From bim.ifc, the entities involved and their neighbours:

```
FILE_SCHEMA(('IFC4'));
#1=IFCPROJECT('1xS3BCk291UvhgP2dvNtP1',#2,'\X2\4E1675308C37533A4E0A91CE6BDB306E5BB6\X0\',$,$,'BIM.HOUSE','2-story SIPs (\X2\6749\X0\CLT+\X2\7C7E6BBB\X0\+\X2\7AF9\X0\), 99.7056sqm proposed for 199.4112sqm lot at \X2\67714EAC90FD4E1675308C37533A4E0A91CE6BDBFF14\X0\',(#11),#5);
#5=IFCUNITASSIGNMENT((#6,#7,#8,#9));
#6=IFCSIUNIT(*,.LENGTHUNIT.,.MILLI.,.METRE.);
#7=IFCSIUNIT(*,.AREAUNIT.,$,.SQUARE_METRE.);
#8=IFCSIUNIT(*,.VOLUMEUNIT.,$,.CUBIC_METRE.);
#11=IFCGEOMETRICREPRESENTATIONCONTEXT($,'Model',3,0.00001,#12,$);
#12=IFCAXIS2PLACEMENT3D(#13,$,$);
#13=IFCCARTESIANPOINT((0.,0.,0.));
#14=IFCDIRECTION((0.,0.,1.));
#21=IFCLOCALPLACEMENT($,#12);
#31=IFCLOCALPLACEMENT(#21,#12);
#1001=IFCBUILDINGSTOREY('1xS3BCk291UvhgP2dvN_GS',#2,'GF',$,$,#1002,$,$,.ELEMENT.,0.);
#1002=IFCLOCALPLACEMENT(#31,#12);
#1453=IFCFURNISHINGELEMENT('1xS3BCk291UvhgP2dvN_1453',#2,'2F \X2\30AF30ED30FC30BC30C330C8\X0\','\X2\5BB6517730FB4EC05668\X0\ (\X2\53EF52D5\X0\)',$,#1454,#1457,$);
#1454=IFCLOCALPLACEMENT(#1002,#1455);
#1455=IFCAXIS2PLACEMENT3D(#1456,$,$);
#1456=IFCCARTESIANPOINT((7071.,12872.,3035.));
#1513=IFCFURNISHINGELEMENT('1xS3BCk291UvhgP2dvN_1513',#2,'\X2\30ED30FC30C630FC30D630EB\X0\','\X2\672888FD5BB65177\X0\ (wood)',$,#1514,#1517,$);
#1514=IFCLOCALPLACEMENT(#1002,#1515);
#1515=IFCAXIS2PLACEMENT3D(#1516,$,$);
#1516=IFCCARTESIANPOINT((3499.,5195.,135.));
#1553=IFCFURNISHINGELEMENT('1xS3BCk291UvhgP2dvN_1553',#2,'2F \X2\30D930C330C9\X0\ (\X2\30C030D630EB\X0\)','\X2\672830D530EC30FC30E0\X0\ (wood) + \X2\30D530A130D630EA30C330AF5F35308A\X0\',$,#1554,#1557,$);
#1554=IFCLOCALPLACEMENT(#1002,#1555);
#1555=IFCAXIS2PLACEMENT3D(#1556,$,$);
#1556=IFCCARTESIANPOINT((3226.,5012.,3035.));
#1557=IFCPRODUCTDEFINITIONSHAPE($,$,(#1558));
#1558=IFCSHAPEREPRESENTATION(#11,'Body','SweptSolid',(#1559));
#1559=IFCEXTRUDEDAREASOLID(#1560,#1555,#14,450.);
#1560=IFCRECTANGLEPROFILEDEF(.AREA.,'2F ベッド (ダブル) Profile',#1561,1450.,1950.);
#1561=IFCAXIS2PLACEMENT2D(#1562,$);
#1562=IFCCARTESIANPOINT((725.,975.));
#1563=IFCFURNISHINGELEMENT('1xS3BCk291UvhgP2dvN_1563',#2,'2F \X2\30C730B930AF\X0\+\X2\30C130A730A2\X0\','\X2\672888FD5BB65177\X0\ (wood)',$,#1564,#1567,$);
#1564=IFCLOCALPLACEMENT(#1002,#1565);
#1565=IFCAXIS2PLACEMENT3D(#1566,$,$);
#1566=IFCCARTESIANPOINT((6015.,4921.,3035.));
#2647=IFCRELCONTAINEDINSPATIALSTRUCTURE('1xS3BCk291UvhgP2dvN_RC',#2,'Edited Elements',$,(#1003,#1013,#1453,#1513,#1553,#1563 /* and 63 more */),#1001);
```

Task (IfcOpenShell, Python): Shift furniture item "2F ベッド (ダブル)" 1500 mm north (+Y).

```python
import ifcopenshell
import ifcopenshell.api.geometry
import ifcopenshell.util.placement

model = ifcopenshell.open("bim.ifc")

item = model.by_id(1553)
matrix = ifcopenshell.util.placement.get_local_placement(item.ObjectPlacement)
matrix[1, 3] += 1500.0
ifcopenshell.api.geometry.edit_object_placement(model, product=item, matrix=matrix, is_si=False)

print(ifcopenshell.util.placement.get_local_placement(item.ObjectPlacement).round(3) + 0.0)

model.write("bim_rev.ifc")
```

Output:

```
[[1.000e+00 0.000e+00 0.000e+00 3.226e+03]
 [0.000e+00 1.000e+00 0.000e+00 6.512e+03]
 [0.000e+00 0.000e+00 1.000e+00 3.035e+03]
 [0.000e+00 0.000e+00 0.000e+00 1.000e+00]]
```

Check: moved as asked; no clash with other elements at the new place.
